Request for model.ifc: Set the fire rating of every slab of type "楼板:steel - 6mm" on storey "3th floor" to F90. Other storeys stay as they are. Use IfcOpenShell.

First a look at what the model holds.

```python
import ifcopenshell
import ifcopenshell.util.element

model = ifcopenshell.open("model.ifc")
print(model.schema)
storey = next(s for s in model.by_type("IfcBuildingStorey") if s.Name == "3th floor")
slabs = [e for e in ifcopenshell.util.element.get_decomposition(storey) if e.is_a("IfcSlab")]
seen = {}
for e in slabs:
    element_type = ifcopenshell.util.element.get_type(e)
    key = (element_type.Name if element_type != e and element_type else None, ifcopenshell.util.element.get_pset(e, "Pset_SlabCommon", "FireRating"))
    seen[key] = seen.get(key, 0) + 1
for (name, value), count in sorted(seen.items(), key=str):
    print(count, "x", name, "|", value)
```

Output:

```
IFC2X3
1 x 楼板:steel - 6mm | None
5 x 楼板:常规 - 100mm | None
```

```python
import ifcopenshell
import ifcopenshell.api.pset
import ifcopenshell.util.element

model = ifcopenshell.open("model.ifc")

storey = next(s for s in model.by_type("IfcBuildingStorey") if s.Name == "3th floor")
slabs = [e for e in ifcopenshell.util.element.get_decomposition(storey) if e.is_a("IfcSlab")]

count = 0
for e in slabs:
    element_type = ifcopenshell.util.element.get_type(e)
    if element_type in (None, e) or element_type.Name != "楼板:steel - 6mm":
        continue
    # add_pset returns the element's existing set when there is one.
    pset = ifcopenshell.api.pset.add_pset(model, product=e, name="Pset_SlabCommon")
    ifcopenshell.api.pset.edit_pset(model, pset=pset, properties={"FireRating": "F90"})
    count += 1

print(count, "slabs updated")

model.write("model_rev.ifc")
```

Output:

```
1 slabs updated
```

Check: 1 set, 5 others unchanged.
